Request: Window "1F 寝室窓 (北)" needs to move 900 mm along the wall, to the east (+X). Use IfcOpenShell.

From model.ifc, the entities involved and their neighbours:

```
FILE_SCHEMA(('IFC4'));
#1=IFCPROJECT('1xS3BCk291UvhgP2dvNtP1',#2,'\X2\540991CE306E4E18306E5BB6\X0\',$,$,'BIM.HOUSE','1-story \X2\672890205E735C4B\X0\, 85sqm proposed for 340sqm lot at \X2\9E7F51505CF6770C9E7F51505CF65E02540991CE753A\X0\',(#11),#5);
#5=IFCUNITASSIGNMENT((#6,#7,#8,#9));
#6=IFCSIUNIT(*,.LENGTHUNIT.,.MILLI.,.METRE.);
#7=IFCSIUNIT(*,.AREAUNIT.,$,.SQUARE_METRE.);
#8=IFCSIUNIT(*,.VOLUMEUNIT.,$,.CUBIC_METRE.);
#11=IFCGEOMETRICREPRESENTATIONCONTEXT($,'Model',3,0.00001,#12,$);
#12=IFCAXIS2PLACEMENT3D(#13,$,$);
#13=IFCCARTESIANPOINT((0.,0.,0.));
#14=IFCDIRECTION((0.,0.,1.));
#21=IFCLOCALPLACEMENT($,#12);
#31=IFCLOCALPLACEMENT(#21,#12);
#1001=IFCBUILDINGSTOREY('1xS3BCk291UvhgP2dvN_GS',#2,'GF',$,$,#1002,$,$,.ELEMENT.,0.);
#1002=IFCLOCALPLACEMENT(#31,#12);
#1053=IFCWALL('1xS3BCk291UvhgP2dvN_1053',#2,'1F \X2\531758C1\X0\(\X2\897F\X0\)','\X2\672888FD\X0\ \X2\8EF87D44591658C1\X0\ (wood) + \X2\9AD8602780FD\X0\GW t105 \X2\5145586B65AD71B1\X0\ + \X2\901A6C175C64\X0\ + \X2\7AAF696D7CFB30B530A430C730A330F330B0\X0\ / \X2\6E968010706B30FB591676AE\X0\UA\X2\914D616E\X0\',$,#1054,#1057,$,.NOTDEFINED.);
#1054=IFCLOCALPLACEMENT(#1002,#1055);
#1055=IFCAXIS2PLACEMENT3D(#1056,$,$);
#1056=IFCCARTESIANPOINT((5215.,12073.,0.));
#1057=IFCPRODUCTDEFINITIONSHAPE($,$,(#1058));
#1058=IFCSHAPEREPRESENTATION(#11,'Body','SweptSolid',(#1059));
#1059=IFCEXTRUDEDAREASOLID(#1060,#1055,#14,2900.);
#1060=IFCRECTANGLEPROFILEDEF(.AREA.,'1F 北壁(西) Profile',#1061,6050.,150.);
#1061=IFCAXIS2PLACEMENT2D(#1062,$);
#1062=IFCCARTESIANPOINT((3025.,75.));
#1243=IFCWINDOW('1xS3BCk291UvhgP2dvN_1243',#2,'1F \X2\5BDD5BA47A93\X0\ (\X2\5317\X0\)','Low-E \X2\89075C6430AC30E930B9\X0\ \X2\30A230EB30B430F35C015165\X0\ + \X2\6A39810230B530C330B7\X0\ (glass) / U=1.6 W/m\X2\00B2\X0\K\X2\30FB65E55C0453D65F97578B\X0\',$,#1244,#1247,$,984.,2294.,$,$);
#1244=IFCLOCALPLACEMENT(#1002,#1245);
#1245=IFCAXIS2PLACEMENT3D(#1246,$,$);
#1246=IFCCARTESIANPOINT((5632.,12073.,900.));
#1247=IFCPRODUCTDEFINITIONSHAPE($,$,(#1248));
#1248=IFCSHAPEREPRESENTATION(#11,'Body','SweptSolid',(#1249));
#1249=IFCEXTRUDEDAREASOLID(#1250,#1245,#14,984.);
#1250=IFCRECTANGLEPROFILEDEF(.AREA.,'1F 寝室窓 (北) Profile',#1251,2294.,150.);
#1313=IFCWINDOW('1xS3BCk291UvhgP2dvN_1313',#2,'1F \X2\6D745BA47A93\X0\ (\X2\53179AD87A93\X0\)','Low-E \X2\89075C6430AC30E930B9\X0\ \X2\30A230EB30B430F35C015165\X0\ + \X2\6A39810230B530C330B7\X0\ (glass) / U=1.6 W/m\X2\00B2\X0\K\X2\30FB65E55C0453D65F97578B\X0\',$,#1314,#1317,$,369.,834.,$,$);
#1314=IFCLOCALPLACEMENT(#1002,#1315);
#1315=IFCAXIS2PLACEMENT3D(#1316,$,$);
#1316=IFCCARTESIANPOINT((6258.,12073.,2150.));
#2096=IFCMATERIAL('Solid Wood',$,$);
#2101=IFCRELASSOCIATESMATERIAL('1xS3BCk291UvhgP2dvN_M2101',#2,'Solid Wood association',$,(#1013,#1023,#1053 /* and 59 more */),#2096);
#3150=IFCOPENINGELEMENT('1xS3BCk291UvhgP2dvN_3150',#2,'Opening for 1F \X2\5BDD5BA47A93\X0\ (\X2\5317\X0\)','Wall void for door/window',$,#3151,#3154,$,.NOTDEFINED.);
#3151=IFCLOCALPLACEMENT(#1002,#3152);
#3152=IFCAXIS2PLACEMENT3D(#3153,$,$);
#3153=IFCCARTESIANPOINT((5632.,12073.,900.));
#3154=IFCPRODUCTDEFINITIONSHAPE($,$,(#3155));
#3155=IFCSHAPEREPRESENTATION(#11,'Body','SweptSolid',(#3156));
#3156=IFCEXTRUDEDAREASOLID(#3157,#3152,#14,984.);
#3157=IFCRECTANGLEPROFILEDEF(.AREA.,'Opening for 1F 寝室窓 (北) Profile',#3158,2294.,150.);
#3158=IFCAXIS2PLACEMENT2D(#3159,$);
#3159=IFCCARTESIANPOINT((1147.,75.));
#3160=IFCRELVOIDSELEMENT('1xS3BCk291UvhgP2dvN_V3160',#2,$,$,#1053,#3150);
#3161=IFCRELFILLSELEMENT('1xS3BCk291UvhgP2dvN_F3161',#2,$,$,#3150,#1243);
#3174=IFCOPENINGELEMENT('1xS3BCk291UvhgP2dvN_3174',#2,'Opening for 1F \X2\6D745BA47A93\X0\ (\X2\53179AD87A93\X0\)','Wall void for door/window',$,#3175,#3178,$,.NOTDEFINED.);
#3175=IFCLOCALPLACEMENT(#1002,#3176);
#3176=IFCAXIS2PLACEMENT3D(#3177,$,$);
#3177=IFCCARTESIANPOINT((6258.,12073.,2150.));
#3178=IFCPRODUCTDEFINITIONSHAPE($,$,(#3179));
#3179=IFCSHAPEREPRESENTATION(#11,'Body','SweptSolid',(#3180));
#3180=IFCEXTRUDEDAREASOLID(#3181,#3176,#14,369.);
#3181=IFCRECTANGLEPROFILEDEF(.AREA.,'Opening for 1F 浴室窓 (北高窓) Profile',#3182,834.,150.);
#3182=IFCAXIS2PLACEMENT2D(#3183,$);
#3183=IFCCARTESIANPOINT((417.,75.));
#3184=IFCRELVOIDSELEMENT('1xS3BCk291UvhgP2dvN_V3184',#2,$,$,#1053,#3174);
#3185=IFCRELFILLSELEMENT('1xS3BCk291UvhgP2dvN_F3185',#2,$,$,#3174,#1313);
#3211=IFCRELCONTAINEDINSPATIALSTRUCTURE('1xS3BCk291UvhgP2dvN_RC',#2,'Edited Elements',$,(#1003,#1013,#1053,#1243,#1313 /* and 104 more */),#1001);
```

```python
import ifcopenshell
import ifcopenshell.api.geometry
import ifcopenshell.util.placement
import ifcopenshell.util.unit

model = ifcopenshell.open("model.ifc")
unit_scale = ifcopenshell.util.unit.calculate_unit_scale(model)

window = model.by_id(1243)
opening = window.FillsVoids[0].RelatingOpeningElement
wall = opening.VoidsElements[0].RelatingBuildingElement

wall_matrix = ifcopenshell.util.placement.get_local_placement(wall.ObjectPlacement)
shift = wall_matrix[:3, 0] * 0.9 / unit_scale
before = ifcopenshell.util.placement.get_local_placement(window.ObjectPlacement)[:3, 3].copy()

# The window is not placed relative to its opening, so move both.
for product in (opening, window):
    matrix = ifcopenshell.util.placement.get_local_placement(product.ObjectPlacement)
    matrix[:3, 3] += shift
    ifcopenshell.api.geometry.edit_object_placement(model, product=product, matrix=matrix, is_si=False)

after = ifcopenshell.util.placement.get_local_placement(window.ObjectPlacement)[:3, 3]
print("window moved by", (after - before).round(3) + 0.0)

model.write("model_updated.ifc")
```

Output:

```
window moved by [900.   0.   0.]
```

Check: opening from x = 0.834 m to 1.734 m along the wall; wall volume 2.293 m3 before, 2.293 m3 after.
